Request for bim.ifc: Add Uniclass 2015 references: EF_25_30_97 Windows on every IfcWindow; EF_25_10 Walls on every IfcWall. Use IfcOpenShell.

First a look at what the model holds.

```python
import ifcopenshell

model = ifcopenshell.open("bim.ifc")
print(model.schema)
print("classifications:", [c.Name for c in model.by_type("IfcClassification")])
for ifc_class in ("IfcDoor", "IfcRoof", "IfcStair", "IfcWall", "IfcWindow"):
    print(ifc_class, len(model.by_type(ifc_class)))
```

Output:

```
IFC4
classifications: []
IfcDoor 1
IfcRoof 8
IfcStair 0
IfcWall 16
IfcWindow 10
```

```python
import ifcopenshell
import ifcopenshell.api.classification

model = ifcopenshell.open("bim.ifc")

system = ifcopenshell.api.classification.add_classification(model, classification="Uniclass 2015")

codes = {
    "IfcWindow": ("EF_25_30_97", "Windows"),
    "IfcWall": ("EF_25_10", "Walls"),
}
for ifc_class, (code, name) in codes.items():
    products = model.by_type(ifc_class)
    ifcopenshell.api.classification.add_reference(
        model, products=products, classification=system, identification=code, name=name
    )
    print(code, len(products))

model.write("bim_rev.ifc")
```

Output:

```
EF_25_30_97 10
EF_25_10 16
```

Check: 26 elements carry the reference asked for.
